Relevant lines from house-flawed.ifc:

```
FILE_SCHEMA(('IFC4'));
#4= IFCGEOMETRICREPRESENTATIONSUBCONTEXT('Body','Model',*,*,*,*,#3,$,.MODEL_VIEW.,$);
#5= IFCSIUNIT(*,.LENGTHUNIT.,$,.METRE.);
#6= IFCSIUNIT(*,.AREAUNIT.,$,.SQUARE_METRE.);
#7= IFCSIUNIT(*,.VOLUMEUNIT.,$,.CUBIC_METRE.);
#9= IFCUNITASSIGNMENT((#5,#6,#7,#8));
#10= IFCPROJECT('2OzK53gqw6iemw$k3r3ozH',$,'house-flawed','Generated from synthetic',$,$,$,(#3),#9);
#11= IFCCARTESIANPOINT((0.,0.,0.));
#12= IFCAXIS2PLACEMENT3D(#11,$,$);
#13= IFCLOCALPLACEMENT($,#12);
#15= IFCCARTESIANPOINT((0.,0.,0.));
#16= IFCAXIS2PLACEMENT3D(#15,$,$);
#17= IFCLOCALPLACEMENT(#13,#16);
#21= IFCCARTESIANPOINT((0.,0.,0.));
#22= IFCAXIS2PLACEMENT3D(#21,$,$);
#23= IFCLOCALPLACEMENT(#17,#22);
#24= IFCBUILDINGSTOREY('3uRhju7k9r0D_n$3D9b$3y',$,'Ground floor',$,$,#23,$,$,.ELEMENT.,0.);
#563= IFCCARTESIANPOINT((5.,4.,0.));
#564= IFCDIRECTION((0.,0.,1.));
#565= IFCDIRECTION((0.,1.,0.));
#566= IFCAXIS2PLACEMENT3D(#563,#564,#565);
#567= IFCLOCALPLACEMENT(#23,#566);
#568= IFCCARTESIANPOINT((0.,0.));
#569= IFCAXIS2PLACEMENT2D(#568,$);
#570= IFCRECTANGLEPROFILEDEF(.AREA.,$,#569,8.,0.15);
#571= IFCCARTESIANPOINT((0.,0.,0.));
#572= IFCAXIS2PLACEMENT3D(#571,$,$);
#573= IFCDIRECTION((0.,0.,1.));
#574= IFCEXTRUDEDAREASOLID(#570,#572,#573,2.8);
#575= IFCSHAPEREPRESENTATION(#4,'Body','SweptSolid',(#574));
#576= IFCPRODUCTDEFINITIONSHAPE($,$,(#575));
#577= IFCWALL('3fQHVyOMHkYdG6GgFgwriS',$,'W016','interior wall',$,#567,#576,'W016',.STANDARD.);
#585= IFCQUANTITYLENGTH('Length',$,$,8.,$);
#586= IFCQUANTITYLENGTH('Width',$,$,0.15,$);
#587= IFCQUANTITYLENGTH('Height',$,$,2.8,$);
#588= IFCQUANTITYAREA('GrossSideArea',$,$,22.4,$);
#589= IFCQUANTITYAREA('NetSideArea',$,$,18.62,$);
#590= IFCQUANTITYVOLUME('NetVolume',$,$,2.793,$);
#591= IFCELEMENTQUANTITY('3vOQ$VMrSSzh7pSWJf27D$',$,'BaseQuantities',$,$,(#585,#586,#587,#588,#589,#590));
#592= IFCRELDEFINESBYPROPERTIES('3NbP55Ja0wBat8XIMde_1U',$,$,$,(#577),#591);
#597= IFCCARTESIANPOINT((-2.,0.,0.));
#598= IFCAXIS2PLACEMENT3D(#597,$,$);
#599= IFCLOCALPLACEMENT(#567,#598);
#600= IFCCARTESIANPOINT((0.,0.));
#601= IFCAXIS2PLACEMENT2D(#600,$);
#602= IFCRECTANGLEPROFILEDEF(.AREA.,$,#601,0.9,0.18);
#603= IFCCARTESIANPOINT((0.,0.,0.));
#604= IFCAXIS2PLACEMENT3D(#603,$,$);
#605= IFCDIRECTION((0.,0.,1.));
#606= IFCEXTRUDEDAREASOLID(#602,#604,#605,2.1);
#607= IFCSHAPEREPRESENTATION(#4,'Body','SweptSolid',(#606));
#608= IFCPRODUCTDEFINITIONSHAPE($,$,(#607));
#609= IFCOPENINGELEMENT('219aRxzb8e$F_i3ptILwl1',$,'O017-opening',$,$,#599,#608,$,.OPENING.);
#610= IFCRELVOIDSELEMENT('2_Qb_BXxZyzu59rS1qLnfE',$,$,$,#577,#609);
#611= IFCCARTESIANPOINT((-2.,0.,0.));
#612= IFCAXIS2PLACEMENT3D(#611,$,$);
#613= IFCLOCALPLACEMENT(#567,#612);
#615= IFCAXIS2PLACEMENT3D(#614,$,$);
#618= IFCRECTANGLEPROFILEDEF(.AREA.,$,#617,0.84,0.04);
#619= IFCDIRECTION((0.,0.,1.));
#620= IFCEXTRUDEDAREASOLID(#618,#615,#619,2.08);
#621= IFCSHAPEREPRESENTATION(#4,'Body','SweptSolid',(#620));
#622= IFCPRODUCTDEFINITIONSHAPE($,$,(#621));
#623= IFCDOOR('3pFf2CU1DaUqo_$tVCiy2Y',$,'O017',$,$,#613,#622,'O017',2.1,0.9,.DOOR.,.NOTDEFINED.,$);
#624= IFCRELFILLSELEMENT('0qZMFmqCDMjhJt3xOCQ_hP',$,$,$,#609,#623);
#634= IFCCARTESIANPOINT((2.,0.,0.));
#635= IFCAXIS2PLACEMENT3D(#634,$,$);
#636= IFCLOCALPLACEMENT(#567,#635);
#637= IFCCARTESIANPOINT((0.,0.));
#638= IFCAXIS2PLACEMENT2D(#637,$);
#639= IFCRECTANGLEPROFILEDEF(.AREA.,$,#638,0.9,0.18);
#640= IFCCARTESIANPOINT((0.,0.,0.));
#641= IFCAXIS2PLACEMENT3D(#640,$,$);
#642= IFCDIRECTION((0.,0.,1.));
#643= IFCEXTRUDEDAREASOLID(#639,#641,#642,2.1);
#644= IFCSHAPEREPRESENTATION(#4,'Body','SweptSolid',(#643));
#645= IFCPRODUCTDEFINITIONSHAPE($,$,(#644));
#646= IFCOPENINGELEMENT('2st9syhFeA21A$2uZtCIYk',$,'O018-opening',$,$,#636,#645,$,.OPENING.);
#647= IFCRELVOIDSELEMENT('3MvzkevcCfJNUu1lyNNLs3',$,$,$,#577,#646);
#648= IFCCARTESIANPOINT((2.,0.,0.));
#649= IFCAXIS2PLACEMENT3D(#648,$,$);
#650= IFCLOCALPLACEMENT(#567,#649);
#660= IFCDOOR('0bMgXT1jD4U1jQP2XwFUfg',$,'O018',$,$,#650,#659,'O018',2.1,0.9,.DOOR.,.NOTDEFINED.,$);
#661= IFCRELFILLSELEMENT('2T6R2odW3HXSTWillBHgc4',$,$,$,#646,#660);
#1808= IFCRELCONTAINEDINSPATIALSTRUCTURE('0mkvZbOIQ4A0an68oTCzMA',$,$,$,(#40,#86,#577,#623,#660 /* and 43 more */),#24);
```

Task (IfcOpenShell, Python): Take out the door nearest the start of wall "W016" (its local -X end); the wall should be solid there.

```python
import ifcopenshell
import ifcopenshell.api.feature
import ifcopenshell.api.pset
import ifcopenshell.api.root
import ifcopenshell.geom
import ifcopenshell.util.element
import ifcopenshell.util.shape
import ifcopenshell.util.unit

model = ifcopenshell.open("house-flawed.ifc")
area_scale = ifcopenshell.util.unit.calculate_unit_scale(model, "AREAUNIT")
volume_scale = ifcopenshell.util.unit.calculate_unit_scale(model, "VOLUMEUNIT")
settings = ifcopenshell.geom.settings()


def volume(element):
    """Net volume in cubic metres, openings subtracted."""
    shape = ifcopenshell.geom.create_shape(settings, element)
    return ifcopenshell.util.shape.get_volume(shape.geometry)


door = model.by_id(623)
opening = door.FillsVoids[0].RelatingOpeningElement
wall = opening.VoidsElements[0].RelatingBuildingElement
before = volume(wall)

ifcopenshell.api.root.remove_product(model, product=door)
ifcopenshell.api.feature.remove_feature(model, feature=opening)

after = volume(wall)
thickness = 0.15  # wall thickness in metres

# Update the wall's stored quantities.
qto = model.by_id(ifcopenshell.util.element.get_pset(wall, "BaseQuantities", should_inherit=False)["id"])
ifcopenshell.api.pset.edit_qto(model, qto=qto, properties={
    "NetSideArea": after / thickness / area_scale,
    "NetVolume": after / volume_scale,
})

print(f"wall volume {before:.3f} -> {after:.3f} m3")

model.write("house-flawed_updated.ifc")
```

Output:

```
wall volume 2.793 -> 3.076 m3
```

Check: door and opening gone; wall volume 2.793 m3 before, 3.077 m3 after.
